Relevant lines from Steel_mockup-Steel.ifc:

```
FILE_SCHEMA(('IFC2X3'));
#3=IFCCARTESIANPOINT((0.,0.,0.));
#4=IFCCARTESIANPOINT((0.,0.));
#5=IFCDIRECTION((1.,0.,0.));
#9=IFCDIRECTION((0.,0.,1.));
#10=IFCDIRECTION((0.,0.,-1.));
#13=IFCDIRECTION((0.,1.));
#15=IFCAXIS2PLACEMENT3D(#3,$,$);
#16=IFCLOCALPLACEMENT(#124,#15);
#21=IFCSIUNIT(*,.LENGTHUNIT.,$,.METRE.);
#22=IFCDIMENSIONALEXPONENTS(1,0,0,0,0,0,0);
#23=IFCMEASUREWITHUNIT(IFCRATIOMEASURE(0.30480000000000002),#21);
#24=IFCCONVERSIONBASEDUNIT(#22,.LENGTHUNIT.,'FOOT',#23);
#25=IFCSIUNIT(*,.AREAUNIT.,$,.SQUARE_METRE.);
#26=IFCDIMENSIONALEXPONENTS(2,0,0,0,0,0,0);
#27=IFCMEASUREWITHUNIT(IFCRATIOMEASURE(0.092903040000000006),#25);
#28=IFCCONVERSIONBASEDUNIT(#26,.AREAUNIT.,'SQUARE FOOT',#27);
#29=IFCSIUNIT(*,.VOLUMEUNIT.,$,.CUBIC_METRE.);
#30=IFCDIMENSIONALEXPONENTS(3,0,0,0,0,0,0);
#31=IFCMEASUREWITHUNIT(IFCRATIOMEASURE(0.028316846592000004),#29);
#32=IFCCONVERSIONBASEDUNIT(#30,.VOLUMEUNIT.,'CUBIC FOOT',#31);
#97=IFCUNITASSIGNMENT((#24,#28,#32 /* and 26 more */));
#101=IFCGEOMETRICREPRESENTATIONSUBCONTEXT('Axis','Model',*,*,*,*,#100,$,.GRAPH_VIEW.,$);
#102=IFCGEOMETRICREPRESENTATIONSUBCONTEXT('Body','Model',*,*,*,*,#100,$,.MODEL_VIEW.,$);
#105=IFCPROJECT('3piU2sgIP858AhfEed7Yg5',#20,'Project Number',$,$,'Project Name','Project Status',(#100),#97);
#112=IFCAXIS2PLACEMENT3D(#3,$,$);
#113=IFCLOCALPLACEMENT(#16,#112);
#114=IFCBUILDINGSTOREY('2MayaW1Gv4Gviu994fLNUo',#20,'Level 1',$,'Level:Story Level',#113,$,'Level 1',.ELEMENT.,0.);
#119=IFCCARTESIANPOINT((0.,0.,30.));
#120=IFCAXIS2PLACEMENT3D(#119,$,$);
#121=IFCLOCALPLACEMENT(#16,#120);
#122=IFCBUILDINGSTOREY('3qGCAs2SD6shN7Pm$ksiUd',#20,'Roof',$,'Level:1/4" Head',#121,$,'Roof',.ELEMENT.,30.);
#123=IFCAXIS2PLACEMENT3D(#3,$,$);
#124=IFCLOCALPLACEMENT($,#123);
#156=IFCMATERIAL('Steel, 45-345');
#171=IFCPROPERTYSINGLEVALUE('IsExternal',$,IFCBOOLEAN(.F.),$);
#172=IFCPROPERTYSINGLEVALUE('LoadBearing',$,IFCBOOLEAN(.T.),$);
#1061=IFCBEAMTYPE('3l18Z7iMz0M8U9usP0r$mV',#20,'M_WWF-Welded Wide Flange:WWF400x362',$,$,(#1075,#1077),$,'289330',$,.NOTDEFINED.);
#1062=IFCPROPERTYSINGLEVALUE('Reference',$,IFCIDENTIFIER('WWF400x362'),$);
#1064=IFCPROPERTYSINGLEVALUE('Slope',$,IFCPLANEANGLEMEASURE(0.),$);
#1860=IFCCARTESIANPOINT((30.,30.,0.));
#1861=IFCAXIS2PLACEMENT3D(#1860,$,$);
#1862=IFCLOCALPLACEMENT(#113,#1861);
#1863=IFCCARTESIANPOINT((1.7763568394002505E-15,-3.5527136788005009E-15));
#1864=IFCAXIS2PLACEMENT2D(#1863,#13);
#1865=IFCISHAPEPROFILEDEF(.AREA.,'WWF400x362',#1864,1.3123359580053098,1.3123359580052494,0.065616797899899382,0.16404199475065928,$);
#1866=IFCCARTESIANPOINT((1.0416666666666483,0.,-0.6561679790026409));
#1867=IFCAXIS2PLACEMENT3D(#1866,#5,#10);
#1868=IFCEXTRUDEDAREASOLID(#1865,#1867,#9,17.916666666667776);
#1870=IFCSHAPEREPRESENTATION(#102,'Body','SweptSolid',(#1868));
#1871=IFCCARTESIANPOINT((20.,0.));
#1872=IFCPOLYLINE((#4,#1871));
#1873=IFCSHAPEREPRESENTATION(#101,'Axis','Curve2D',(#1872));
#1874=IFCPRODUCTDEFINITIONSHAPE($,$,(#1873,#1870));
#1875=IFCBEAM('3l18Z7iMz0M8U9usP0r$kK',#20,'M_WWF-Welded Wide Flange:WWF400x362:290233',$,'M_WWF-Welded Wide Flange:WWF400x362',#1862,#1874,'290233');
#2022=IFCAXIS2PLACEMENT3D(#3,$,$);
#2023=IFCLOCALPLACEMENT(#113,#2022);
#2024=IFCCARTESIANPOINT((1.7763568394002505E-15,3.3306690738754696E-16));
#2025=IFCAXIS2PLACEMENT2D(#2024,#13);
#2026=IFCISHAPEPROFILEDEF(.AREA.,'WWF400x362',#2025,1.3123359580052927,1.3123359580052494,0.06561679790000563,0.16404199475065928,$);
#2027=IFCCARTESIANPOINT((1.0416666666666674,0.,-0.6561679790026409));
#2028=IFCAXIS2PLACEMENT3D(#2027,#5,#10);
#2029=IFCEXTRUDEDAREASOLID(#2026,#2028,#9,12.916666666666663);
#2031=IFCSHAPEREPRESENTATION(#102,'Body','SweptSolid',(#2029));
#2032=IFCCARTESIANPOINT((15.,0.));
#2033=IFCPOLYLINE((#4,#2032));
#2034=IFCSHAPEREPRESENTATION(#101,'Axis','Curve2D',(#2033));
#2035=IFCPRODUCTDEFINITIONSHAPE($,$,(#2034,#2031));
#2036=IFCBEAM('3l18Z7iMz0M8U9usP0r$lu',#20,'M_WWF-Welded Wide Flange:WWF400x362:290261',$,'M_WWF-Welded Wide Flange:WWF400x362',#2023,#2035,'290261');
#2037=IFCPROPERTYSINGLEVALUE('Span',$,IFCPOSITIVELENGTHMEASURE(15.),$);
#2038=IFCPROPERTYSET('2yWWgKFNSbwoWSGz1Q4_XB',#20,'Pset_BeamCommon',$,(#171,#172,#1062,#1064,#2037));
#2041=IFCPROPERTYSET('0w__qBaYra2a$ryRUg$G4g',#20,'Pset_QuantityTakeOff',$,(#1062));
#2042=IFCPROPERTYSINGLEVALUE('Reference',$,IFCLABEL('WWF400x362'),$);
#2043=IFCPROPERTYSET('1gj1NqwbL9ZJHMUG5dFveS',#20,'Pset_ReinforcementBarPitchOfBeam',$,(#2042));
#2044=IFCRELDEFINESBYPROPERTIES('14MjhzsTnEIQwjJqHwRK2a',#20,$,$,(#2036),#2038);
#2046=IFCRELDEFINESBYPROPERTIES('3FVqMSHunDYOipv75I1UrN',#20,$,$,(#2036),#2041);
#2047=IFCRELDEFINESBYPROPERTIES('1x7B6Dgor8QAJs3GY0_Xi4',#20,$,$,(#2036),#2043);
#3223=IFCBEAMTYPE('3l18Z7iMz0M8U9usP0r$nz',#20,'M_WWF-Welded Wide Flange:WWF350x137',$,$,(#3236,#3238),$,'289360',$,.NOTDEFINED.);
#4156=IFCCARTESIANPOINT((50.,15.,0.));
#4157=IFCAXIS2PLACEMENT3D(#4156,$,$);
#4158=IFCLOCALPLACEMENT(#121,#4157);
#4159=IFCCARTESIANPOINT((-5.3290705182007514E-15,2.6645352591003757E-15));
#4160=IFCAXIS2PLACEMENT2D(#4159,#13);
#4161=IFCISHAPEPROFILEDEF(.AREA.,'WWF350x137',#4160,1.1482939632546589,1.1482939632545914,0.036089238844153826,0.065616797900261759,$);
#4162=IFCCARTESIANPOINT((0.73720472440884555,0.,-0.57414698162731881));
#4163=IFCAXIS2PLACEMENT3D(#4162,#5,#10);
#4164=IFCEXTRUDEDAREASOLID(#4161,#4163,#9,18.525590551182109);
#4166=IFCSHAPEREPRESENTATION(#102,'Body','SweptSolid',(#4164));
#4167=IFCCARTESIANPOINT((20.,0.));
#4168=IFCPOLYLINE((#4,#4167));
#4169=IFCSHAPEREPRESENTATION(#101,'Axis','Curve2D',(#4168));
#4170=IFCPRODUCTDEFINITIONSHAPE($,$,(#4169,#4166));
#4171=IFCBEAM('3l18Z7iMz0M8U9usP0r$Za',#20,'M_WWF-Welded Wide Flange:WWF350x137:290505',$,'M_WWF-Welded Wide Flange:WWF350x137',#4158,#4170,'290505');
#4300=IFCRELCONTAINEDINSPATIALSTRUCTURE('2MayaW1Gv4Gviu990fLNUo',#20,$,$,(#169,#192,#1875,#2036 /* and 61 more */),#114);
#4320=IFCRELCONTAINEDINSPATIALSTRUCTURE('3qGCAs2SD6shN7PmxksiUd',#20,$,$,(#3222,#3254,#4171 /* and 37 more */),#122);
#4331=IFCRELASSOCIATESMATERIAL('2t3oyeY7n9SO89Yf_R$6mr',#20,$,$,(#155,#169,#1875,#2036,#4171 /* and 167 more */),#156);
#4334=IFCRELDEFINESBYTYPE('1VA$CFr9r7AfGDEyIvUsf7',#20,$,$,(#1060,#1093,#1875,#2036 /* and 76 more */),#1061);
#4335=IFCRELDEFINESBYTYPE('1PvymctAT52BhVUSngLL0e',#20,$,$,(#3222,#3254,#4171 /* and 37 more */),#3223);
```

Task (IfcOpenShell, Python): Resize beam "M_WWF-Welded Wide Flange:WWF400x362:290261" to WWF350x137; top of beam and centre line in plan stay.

```python
import ifcopenshell
import ifcopenshell.api.pset
import ifcopenshell.api.type
import ifcopenshell.util.element
import ifcopenshell.util.representation

model = ifcopenshell.open("Steel_mockup-Steel.ifc")

member = model.by_guid("3l18Z7iMz0M8U9usP0r$lu")
source = next(p for p in model.by_type("IfcIShapeProfileDef") if p.ProfileName == "WWF350x137")

body = ifcopenshell.util.representation.get_representation(member, "Model", "Body")
solid = body.Items[0]
old_profile = solid.SweptArea

# Copy the section's sizes but keep this member's own profile position.
profile = ifcopenshell.util.element.copy(model, source)
# Profiles are centred, so shift by half the change in depth to hold the top.
shift = (old_profile.OverallDepth - profile.OverallDepth) / 2
x, y = old_profile.Position.Location.Coordinates
up = (-1.0, 0.0)  # upwards, in the solid's own plane
location = model.createIfcCartesianPoint((x + up[0] * shift, y + up[1] * shift))
profile.Position = model.createIfcAxis2Placement2D(location, old_profile.Position.RefDirection)
solid.SweptArea = profile
if not model.get_total_inverses(old_profile):
    ifcopenshell.util.element.remove_deep2(model, old_profile)

new_type = model.by_guid("3l18Z7iMz0M8U9usP0r$nz")
ifcopenshell.api.type.assign_type(
    model, related_objects=[member], relating_type=new_type, should_map_representations=False
)
member.Name = member.Name.replace("WWF400x362", "WWF350x137")
member.ObjectType = "M_WWF-Welded Wide Flange:WWF350x137"
pset = model.by_id(ifcopenshell.util.element.get_pset(member, "Pset_BeamCommon", should_inherit=False)["id"])
ifcopenshell.api.pset.edit_pset(model, pset=pset, properties={"Reference": "WWF350x137"})
pset = model.by_id(ifcopenshell.util.element.get_pset(member, "Pset_QuantityTakeOff", should_inherit=False)["id"])
ifcopenshell.api.pset.edit_pset(model, pset=pset, properties={"Reference": "WWF350x137"})
pset = model.by_id(ifcopenshell.util.element.get_pset(member, "Pset_ReinforcementBarPitchOfBeam", should_inherit=False)["id"])
ifcopenshell.api.pset.edit_pset(model, pset=pset, properties={"Reference": "WWF350x137"})

print(solid.SweptArea)

model.write("Steel_mockup-Steel_v2.ifc")
```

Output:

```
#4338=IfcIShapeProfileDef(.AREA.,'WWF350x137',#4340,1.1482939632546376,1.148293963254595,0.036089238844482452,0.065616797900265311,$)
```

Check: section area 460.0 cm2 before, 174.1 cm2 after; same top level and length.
